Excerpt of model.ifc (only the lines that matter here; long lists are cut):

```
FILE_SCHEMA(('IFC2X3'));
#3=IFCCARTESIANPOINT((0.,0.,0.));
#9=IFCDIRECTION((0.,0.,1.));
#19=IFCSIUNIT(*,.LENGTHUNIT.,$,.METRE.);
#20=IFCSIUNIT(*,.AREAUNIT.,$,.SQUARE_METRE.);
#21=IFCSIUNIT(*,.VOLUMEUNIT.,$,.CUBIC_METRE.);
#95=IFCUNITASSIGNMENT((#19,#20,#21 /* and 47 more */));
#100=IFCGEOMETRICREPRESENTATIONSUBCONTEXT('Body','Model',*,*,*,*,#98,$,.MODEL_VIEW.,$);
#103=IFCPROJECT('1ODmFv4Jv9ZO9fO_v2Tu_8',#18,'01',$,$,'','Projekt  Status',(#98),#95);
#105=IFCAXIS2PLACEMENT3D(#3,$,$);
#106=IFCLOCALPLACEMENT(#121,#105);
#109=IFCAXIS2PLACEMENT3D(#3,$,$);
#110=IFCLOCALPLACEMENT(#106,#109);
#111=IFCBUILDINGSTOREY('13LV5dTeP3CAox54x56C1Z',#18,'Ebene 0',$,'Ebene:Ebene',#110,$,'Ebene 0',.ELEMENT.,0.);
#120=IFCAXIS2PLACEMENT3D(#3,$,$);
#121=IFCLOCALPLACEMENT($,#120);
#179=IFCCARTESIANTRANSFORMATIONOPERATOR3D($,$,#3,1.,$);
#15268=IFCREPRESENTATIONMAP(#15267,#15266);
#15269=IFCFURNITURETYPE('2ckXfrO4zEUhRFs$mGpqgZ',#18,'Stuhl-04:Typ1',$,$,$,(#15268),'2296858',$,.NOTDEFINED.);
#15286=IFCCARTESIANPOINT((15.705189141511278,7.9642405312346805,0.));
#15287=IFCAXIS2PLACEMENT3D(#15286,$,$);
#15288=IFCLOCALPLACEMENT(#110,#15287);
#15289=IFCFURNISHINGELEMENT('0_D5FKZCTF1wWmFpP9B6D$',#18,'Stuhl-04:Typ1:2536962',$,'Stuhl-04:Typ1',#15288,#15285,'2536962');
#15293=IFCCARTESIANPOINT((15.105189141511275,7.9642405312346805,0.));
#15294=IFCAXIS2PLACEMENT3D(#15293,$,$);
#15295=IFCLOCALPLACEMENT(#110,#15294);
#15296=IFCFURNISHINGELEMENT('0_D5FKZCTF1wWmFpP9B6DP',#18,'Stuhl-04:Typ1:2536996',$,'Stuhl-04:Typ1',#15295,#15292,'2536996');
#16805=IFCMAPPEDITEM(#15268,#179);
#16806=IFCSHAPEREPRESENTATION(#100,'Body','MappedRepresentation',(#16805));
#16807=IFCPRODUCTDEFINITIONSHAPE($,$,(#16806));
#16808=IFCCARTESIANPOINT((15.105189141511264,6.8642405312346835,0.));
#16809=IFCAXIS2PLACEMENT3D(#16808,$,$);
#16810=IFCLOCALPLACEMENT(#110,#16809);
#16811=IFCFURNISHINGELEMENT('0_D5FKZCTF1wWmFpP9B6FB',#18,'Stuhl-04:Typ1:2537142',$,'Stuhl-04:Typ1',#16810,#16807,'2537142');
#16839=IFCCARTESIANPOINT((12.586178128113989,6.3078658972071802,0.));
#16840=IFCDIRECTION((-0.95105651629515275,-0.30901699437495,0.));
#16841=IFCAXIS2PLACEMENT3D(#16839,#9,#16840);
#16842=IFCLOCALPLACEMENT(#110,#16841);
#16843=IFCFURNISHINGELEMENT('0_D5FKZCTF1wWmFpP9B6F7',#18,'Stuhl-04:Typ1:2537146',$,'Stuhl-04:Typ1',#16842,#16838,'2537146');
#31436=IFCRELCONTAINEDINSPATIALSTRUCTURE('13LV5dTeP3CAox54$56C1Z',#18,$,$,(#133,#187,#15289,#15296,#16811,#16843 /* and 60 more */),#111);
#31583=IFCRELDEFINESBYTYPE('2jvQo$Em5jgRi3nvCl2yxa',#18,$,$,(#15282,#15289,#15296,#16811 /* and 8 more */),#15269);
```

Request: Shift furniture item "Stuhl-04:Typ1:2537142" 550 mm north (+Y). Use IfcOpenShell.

```python
import ifcopenshell
import ifcopenshell.api.geometry
import ifcopenshell.util.placement
import ifcopenshell.util.unit

model = ifcopenshell.open("model.ifc")
unit_scale = ifcopenshell.util.unit.calculate_unit_scale(model)

item = model.by_id(16811)
matrix = ifcopenshell.util.placement.get_local_placement(item.ObjectPlacement)
matrix[1, 3] += 0.55 / unit_scale
ifcopenshell.api.geometry.edit_object_placement(model, product=item, matrix=matrix, is_si=False)

print(ifcopenshell.util.placement.get_local_placement(item.ObjectPlacement).round(3) + 0.0)

model.write("model_updated.ifc")
```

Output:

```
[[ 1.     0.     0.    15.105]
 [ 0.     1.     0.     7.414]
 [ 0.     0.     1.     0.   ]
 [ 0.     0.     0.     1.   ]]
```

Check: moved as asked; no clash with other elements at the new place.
